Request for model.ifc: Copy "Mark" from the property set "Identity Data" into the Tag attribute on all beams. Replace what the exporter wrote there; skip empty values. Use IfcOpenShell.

First a look at what the model holds.

```python
import ifcopenshell
import ifcopenshell.util.element

model = ifcopenshell.open("model.ifc")
print(model.schema)
beams = model.by_type("IfcBeam")
print(len(beams), "beams")
for e in beams[:8]:
    source = ifcopenshell.util.element.get_pset(e, "Identity Data", "Mark")
    target = e.Tag
    print(e.id(), repr(source), repr(target), sep=" | ")
```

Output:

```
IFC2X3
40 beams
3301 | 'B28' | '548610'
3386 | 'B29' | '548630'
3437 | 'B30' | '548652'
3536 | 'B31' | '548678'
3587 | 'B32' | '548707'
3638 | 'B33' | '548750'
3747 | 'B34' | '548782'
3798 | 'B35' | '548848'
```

```python
import ifcopenshell
import ifcopenshell.util.element

model = ifcopenshell.open("model.ifc")

count = 0
for e in model.by_type("IfcBeam"):
    value = ifcopenshell.util.element.get_pset(e, "Identity Data", "Mark")
    current = e.Tag
    if not value or not value.strip() or current == value:
        continue
    e.Tag = value
    count += 1

print(count, "beams updated")

model.write("model-out.ifc")
```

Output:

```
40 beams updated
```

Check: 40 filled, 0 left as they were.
